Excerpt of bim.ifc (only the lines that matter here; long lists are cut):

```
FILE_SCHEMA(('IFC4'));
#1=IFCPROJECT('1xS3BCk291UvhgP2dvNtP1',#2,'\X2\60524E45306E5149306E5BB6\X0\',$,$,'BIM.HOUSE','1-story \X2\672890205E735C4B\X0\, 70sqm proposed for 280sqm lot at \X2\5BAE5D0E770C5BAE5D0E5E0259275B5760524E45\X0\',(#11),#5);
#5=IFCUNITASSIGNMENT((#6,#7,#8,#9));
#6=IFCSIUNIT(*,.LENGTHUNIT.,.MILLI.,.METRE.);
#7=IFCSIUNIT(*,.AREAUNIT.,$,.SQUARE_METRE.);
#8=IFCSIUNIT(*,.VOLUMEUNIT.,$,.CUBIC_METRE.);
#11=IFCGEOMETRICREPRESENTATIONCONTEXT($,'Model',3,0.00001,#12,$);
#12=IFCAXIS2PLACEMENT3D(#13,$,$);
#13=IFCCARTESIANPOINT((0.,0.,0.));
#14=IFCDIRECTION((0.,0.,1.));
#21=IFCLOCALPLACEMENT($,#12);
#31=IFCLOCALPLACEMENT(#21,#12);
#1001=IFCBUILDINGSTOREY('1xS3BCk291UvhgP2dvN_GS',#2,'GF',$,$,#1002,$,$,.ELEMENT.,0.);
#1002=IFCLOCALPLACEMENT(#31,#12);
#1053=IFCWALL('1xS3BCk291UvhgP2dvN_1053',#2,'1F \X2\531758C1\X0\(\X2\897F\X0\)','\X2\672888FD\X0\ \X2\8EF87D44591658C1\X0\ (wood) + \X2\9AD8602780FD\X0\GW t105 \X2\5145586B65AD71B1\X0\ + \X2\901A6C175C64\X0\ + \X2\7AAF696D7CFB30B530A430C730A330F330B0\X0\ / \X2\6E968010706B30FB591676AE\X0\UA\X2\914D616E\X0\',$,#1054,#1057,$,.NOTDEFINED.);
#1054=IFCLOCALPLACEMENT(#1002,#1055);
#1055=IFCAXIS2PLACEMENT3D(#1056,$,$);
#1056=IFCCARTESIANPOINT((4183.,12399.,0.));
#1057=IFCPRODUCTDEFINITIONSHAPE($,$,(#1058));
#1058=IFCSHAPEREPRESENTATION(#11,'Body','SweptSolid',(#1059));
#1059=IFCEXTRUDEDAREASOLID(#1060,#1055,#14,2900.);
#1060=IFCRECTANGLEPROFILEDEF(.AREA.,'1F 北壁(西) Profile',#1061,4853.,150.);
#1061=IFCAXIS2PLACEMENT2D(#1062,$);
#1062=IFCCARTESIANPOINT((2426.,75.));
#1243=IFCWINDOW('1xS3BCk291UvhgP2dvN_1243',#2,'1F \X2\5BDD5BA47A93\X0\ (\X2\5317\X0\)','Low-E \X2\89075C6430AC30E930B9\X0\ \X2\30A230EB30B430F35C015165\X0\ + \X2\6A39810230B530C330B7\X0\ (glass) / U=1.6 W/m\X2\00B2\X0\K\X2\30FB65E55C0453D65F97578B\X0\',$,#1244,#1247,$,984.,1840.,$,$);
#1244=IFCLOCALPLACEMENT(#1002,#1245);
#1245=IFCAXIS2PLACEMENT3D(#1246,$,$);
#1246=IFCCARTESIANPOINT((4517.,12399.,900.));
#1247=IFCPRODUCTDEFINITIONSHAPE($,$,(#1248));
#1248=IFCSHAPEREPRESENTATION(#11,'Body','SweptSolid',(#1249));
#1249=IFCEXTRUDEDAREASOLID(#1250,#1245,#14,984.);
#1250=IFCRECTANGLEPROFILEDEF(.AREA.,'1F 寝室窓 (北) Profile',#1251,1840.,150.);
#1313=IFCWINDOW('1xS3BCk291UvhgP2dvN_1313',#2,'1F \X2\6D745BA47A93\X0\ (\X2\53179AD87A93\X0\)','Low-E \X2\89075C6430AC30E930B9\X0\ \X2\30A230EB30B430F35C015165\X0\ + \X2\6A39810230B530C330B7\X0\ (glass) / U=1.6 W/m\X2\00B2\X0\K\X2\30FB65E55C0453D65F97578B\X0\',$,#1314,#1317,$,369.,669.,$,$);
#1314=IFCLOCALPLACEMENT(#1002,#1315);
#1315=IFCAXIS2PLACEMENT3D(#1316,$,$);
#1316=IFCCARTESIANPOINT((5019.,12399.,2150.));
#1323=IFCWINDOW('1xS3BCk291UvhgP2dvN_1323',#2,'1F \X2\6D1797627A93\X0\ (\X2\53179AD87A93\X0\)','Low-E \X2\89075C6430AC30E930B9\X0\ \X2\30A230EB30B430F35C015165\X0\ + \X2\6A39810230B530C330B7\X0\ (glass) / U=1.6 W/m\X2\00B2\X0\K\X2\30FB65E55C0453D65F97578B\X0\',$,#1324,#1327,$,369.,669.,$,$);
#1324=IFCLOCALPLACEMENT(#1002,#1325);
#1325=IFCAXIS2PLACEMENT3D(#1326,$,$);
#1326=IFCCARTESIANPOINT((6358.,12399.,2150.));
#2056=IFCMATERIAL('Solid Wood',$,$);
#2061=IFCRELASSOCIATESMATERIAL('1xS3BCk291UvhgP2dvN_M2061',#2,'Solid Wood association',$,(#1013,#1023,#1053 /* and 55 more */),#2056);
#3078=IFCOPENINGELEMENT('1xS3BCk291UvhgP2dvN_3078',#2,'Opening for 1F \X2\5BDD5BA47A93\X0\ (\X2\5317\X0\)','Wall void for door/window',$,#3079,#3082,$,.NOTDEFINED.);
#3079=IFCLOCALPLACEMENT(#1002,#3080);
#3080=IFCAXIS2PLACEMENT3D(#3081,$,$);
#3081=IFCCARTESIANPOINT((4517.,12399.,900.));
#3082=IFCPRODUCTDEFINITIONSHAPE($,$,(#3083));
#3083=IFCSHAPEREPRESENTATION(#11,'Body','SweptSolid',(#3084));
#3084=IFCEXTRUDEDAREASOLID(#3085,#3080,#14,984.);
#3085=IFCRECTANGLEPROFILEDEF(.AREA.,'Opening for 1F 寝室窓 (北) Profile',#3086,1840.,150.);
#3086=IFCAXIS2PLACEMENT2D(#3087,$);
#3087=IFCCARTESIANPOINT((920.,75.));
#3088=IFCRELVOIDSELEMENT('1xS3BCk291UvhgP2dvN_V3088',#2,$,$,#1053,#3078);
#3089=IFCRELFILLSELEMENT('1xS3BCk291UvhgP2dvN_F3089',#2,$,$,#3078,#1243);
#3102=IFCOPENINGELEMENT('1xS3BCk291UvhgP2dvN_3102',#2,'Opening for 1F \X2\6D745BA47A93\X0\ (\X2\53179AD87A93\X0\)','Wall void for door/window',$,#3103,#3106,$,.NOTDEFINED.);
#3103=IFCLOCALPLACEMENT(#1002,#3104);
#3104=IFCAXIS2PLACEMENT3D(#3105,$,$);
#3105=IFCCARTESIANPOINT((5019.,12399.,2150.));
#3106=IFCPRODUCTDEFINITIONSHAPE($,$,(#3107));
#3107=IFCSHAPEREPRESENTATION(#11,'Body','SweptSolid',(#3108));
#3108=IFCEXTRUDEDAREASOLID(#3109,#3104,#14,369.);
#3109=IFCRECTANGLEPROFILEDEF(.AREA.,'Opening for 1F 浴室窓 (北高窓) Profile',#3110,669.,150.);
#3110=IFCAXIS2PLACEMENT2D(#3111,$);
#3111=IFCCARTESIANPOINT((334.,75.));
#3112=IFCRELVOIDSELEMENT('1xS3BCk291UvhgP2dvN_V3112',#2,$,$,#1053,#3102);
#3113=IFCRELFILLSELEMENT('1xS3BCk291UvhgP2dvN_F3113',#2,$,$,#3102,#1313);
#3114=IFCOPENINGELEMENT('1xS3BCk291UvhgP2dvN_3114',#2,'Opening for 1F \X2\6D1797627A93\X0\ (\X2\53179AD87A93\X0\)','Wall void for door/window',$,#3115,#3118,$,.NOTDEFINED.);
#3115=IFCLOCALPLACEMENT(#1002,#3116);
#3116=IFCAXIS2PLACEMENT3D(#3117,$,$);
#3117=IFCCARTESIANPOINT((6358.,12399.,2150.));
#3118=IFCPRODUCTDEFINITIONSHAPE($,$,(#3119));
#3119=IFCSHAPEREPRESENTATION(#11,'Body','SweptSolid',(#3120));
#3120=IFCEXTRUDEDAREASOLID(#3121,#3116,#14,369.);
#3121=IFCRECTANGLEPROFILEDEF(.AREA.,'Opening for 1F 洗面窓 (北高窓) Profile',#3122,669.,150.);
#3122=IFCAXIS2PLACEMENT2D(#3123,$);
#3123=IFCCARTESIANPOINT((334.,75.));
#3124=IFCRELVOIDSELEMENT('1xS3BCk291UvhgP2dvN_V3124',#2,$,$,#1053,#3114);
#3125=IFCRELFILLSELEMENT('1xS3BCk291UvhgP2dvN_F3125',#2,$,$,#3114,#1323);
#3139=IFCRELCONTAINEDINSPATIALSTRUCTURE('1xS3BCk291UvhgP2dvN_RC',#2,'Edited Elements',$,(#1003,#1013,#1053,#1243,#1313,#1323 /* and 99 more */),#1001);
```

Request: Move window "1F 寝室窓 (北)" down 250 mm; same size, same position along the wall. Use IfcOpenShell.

```python
import numpy as np
import ifcopenshell
import ifcopenshell.api.geometry
import ifcopenshell.util.placement
import ifcopenshell.util.unit

model = ifcopenshell.open("bim.ifc")
unit_scale = ifcopenshell.util.unit.calculate_unit_scale(model)

window = model.by_id(1243)
opening = window.FillsVoids[0].RelatingOpeningElement
dz = -0.25 / unit_scale

shift = np.array([0.0, 0.0, dz])
# The window is not placed relative to its opening, so move both.
for product in (opening, window):
    matrix = ifcopenshell.util.placement.get_local_placement(product.ObjectPlacement)
    matrix[:3, 3] += shift
    ifcopenshell.api.geometry.edit_object_placement(model, product=product, matrix=matrix, is_si=False)

print(f"moved by {dz * unit_scale:+.3f} m")

model.write("bim_edited.ifc")
```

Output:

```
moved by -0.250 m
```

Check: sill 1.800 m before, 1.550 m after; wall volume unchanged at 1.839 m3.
